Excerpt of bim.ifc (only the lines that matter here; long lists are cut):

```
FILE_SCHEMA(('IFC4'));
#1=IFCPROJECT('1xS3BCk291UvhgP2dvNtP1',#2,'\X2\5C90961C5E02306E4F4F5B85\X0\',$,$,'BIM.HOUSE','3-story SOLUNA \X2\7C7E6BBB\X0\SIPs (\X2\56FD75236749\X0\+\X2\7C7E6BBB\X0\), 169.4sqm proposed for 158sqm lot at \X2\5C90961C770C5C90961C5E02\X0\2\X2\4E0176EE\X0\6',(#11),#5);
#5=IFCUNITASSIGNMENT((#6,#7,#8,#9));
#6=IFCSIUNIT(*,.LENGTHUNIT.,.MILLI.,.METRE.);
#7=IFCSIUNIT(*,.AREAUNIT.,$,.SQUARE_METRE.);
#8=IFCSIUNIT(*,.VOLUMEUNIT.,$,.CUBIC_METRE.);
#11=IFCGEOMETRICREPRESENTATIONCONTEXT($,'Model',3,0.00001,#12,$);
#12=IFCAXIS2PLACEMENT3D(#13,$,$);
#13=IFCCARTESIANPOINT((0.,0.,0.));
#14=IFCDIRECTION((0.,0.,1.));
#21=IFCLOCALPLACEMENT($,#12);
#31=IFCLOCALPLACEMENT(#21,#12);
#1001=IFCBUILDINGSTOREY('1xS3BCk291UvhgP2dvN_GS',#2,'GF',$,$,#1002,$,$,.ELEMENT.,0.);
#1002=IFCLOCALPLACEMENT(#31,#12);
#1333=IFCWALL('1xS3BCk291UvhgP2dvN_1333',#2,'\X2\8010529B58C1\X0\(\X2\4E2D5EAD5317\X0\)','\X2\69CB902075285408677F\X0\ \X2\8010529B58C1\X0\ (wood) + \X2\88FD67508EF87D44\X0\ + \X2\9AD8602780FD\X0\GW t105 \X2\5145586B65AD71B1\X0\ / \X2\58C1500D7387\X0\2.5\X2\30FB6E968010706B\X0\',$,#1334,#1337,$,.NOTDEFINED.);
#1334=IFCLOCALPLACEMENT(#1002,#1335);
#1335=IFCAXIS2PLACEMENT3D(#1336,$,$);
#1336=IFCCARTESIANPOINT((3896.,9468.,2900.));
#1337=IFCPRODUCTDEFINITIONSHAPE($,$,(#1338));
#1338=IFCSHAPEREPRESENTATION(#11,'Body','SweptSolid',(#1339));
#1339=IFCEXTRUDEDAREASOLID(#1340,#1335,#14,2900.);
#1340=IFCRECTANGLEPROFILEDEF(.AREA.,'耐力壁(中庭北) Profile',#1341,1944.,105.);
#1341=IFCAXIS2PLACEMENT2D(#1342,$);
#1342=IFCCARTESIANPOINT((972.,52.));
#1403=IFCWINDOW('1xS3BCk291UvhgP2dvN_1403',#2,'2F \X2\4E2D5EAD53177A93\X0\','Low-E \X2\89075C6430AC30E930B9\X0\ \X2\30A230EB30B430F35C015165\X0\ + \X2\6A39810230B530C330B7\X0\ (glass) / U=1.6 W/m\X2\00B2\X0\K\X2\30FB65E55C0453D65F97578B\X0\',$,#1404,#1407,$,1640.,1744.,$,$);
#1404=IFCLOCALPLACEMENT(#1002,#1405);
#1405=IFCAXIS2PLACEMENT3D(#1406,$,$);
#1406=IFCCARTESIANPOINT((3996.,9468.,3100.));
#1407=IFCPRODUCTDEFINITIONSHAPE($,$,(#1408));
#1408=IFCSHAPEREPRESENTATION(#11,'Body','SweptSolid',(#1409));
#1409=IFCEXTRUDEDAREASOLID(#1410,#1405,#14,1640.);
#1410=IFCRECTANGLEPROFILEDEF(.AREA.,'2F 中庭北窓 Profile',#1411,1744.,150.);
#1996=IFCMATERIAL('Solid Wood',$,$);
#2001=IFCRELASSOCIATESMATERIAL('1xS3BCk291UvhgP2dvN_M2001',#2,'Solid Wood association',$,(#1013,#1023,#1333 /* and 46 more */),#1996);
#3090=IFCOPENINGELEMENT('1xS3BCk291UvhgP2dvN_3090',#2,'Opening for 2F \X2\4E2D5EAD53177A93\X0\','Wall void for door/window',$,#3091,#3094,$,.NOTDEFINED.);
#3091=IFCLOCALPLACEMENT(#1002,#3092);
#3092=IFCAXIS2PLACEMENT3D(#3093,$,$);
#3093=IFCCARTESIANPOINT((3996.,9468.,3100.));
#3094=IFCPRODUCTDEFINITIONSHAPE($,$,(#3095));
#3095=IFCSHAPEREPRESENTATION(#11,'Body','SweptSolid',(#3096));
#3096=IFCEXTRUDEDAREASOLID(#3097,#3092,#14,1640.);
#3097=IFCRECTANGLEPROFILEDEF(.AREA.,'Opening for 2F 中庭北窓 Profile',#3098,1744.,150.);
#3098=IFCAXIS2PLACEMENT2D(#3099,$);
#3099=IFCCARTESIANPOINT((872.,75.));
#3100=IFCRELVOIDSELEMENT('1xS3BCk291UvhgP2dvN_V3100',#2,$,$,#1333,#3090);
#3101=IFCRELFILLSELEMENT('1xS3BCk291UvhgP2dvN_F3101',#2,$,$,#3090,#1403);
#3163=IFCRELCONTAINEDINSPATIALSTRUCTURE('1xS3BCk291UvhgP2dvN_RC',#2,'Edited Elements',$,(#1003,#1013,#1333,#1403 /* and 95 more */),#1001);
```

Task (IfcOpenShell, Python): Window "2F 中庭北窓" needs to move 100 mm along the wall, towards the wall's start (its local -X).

```python
import ifcopenshell
import ifcopenshell.api.geometry
import ifcopenshell.util.placement
import ifcopenshell.util.unit

model = ifcopenshell.open("bim.ifc")
unit_scale = ifcopenshell.util.unit.calculate_unit_scale(model)

window = model.by_guid("1xS3BCk291UvhgP2dvN_1403")
opening = window.FillsVoids[0].RelatingOpeningElement
wall = opening.VoidsElements[0].RelatingBuildingElement

wall_matrix = ifcopenshell.util.placement.get_local_placement(wall.ObjectPlacement)
shift = wall_matrix[:3, 0] * -0.1 / unit_scale
before = ifcopenshell.util.placement.get_local_placement(window.ObjectPlacement)[:3, 3].copy()

# The window is not placed relative to its opening, so move both.
for product in (opening, window):
    matrix = ifcopenshell.util.placement.get_local_placement(product.ObjectPlacement)
    matrix[:3, 3] += shift
    ifcopenshell.api.geometry.edit_object_placement(model, product=product, matrix=matrix, is_si=False)

after = ifcopenshell.util.placement.get_local_placement(window.ObjectPlacement)[:3, 3]
print("window moved by", (after - before).round(3) + 0.0)

model.write("bim_updated.ifc")
```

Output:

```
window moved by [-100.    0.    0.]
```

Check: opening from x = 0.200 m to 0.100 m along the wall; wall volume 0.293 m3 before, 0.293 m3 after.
